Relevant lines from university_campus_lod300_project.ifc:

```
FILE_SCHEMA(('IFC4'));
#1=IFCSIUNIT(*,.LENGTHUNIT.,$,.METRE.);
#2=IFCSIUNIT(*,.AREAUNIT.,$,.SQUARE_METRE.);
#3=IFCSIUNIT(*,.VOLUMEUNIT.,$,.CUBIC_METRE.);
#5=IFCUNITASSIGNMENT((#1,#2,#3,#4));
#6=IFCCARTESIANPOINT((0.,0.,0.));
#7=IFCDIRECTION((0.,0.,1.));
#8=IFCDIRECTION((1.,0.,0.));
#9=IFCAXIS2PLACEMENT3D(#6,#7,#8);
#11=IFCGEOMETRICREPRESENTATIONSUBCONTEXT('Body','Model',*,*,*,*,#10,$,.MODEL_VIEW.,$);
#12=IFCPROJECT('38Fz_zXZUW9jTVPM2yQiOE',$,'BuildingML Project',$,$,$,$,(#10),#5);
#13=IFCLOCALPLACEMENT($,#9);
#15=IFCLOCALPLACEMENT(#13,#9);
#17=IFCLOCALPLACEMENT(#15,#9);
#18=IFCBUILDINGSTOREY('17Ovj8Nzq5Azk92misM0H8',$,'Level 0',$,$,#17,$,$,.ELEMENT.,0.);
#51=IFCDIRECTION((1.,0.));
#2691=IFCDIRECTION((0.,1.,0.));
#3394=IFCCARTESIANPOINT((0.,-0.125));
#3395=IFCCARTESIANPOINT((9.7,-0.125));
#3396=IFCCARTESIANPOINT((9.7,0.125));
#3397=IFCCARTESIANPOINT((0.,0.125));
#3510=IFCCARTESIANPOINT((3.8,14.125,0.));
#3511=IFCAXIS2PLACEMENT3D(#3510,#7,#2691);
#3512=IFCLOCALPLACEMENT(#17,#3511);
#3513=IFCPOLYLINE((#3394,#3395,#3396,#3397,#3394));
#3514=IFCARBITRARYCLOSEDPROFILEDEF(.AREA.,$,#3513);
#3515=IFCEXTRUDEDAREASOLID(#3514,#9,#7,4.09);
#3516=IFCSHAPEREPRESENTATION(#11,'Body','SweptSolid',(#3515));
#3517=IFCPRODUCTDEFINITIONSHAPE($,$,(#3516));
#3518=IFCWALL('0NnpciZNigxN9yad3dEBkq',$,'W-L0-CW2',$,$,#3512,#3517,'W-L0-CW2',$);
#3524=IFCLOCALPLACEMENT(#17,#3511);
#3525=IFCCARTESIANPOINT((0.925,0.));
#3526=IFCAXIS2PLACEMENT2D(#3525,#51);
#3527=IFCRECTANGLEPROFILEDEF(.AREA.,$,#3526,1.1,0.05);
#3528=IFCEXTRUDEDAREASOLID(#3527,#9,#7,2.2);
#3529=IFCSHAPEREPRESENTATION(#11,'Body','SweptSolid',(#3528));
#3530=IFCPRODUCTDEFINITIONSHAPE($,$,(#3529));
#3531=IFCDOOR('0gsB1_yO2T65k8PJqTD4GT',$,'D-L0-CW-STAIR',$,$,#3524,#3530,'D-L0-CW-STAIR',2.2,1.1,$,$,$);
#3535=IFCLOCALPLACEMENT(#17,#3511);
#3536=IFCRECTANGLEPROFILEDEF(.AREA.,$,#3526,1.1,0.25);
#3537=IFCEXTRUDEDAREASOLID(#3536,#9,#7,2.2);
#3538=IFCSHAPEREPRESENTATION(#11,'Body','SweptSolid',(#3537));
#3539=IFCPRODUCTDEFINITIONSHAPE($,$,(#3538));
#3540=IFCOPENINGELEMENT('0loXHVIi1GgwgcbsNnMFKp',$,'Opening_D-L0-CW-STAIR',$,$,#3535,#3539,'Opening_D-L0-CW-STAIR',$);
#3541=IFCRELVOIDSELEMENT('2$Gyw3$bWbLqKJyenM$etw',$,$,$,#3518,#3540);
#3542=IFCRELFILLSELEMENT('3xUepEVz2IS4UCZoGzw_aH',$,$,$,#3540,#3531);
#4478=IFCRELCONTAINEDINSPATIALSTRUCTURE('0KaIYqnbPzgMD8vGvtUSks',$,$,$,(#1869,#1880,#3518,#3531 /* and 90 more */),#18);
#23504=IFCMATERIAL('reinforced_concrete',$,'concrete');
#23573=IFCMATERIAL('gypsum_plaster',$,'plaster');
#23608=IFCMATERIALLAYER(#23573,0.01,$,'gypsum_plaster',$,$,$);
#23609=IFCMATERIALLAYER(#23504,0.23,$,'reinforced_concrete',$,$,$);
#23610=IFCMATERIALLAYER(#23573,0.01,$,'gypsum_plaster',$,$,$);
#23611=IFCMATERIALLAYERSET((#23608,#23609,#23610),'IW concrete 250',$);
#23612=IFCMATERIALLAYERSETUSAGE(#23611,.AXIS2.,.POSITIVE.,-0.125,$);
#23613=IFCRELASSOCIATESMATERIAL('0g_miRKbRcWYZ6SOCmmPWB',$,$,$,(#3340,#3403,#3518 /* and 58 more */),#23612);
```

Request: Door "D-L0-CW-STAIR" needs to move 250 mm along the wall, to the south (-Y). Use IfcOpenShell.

```python
import ifcopenshell
import ifcopenshell.api.geometry
import ifcopenshell.util.placement
import ifcopenshell.util.unit

model = ifcopenshell.open("university_campus_lod300_project.ifc")
unit_scale = ifcopenshell.util.unit.calculate_unit_scale(model)

door = model.by_id(3531)
opening = door.FillsVoids[0].RelatingOpeningElement
wall = opening.VoidsElements[0].RelatingBuildingElement

wall_matrix = ifcopenshell.util.placement.get_local_placement(wall.ObjectPlacement)
shift = wall_matrix[:3, 0] * -0.25 / unit_scale
before = ifcopenshell.util.placement.get_local_placement(door.ObjectPlacement)[:3, 3].copy()

# The door is not placed relative to its opening, so move both.
for product in (opening, door):
    matrix = ifcopenshell.util.placement.get_local_placement(product.ObjectPlacement)
    matrix[:3, 3] += shift
    ifcopenshell.api.geometry.edit_object_placement(model, product=product, matrix=matrix, is_si=False)

after = ifcopenshell.util.placement.get_local_placement(door.ObjectPlacement)[:3, 3]
print("door moved by", (after - before).round(3) + 0.0)

model.write("university_campus_lod300_project_v2.ifc")
```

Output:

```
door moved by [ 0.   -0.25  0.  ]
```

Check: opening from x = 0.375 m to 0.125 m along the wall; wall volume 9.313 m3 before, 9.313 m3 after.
